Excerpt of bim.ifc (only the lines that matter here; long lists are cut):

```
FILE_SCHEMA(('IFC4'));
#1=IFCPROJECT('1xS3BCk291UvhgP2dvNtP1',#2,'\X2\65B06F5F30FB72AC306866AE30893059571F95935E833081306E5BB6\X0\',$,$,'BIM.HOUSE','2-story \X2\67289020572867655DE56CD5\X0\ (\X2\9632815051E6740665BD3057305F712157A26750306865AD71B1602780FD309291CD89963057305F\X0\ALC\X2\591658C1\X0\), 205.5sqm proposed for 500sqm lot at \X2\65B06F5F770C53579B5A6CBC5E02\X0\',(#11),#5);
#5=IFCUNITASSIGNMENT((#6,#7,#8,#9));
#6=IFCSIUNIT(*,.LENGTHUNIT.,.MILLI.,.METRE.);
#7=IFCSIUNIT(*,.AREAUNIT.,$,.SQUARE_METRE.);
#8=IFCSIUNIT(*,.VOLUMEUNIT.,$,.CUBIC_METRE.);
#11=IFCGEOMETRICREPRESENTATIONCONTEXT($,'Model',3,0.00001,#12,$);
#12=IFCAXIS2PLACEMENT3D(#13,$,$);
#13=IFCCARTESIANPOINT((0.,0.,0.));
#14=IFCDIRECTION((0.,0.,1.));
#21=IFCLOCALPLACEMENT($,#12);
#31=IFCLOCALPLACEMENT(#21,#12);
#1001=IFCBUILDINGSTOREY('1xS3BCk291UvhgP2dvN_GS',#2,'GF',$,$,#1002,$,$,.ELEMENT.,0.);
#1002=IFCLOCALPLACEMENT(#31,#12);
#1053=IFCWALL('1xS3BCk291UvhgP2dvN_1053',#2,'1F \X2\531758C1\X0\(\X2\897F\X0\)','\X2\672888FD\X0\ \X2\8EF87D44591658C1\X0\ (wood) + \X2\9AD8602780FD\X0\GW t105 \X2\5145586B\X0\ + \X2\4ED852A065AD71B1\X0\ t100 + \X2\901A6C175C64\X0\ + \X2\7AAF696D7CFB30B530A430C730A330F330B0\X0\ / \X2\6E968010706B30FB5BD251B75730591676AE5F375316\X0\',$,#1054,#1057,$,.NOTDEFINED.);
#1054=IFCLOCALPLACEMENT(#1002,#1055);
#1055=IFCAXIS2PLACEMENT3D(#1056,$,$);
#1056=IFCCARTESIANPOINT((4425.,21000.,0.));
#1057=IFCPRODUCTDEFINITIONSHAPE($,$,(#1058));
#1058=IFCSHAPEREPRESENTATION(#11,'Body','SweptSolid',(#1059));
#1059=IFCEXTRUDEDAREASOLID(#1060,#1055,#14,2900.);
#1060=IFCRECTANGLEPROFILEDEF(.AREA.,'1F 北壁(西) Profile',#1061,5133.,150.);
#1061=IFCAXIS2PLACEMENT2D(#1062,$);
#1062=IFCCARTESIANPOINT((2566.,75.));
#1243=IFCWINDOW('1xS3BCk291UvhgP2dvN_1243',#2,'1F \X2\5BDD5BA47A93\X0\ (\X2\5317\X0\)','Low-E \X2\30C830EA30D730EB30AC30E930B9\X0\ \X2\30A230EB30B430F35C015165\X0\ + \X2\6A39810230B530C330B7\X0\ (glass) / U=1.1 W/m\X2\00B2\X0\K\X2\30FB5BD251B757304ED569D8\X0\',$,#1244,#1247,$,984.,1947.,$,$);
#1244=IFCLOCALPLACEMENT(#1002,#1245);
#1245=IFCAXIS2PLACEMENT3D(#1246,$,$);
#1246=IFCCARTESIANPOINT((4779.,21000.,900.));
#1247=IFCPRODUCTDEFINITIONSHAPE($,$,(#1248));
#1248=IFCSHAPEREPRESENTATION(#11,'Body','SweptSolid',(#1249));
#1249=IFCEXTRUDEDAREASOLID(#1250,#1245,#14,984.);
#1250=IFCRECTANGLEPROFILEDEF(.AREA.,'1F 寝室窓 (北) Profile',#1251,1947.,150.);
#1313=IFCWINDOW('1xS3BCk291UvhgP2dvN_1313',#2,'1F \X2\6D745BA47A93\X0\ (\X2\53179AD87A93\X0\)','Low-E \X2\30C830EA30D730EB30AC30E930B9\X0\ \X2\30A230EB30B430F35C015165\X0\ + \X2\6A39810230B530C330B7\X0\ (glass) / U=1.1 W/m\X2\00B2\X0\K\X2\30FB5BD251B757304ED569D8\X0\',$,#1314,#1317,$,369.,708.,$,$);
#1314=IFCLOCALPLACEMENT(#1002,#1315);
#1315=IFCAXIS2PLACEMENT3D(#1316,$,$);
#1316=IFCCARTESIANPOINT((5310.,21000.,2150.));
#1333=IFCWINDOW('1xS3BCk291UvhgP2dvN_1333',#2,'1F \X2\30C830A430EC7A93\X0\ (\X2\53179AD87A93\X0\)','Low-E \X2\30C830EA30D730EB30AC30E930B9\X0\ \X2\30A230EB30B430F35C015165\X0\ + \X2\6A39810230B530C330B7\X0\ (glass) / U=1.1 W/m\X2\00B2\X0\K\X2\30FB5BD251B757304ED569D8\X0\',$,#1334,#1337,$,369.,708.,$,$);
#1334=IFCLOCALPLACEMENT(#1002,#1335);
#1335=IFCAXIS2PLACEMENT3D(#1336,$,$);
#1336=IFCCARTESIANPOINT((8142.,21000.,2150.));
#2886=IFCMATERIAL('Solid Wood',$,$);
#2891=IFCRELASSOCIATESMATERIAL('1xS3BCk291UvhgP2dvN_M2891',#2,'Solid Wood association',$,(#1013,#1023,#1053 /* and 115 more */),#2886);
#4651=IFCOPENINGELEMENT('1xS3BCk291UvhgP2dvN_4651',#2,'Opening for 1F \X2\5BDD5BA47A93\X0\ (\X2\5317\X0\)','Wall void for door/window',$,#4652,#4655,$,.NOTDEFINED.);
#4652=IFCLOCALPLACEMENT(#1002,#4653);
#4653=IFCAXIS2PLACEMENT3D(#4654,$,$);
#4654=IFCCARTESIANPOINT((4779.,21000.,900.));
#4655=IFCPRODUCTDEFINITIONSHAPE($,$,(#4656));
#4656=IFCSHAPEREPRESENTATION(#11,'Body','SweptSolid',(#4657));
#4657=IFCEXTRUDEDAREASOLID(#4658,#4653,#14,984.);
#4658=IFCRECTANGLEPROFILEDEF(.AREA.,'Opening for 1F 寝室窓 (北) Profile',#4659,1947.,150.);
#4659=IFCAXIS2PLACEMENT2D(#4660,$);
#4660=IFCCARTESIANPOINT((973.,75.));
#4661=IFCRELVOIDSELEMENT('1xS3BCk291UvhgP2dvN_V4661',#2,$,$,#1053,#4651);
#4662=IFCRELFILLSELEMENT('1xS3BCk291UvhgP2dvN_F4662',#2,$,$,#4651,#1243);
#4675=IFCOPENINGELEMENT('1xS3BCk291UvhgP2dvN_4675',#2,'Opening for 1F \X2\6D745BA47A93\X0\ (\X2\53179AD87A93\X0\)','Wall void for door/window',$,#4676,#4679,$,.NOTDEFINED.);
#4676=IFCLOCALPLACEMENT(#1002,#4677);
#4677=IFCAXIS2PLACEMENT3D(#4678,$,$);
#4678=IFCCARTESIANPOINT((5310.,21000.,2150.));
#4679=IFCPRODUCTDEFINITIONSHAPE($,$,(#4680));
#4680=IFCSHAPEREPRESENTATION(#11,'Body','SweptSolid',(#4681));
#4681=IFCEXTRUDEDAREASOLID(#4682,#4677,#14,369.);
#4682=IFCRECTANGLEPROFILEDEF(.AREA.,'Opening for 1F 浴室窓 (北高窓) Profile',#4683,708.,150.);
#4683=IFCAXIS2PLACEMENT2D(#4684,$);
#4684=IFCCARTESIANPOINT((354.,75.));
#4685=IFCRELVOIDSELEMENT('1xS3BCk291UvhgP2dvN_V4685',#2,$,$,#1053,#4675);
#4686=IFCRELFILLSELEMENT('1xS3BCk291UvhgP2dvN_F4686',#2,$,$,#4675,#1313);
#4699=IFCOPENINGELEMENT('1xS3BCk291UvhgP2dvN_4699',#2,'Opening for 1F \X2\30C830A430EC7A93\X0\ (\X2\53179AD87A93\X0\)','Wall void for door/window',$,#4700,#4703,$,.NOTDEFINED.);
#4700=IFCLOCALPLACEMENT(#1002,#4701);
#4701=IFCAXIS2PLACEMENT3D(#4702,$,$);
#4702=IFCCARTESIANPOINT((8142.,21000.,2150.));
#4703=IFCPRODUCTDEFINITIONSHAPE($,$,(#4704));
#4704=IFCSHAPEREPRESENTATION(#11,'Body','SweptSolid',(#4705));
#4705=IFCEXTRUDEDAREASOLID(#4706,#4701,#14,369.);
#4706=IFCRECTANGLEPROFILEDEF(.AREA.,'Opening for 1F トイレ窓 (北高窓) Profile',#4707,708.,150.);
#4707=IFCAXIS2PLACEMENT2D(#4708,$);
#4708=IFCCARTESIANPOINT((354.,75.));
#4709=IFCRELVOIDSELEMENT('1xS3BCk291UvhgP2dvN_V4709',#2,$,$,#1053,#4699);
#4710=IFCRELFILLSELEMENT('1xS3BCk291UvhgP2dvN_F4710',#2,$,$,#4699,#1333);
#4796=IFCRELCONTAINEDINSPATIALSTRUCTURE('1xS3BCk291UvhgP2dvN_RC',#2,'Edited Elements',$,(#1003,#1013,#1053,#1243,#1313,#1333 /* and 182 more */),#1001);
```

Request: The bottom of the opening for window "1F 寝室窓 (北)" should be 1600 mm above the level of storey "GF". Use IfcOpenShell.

```python
import numpy as np
import ifcopenshell
import ifcopenshell.api.geometry
import ifcopenshell.geom
import ifcopenshell.util.element
import ifcopenshell.util.placement
import ifcopenshell.util.shape
import ifcopenshell.util.unit

model = ifcopenshell.open("bim.ifc")
unit_scale = ifcopenshell.util.unit.calculate_unit_scale(model)

window = model.by_guid("1xS3BCk291UvhgP2dvN_1243")
opening = window.FillsVoids[0].RelatingOpeningElement
storey = ifcopenshell.util.element.get_container(window, ifc_class="IfcBuildingStorey")
level = ifcopenshell.util.placement.get_local_placement(storey.ObjectPlacement)[2, 3]

# The opening's origin need not be at the sill, so measure its lowest point.
shape = ifcopenshell.geom.create_shape(ifcopenshell.geom.settings(), opening)
bottom = ifcopenshell.util.shape.get_shape_bottom_elevation(shape, shape.geometry) / unit_scale
dz = level + 1.6 / unit_scale - bottom

shift = np.array([0.0, 0.0, dz])
# The window is not placed relative to its opening, so move both.
for product in (opening, window):
    matrix = ifcopenshell.util.placement.get_local_placement(product.ObjectPlacement)
    matrix[:3, 3] += shift
    ifcopenshell.api.geometry.edit_object_placement(model, product=product, matrix=matrix, is_si=False)

print(f"moved by {dz * unit_scale:+.3f} m")

model.write("bim_updated.ifc")
```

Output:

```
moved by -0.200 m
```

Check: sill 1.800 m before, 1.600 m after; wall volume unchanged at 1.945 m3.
